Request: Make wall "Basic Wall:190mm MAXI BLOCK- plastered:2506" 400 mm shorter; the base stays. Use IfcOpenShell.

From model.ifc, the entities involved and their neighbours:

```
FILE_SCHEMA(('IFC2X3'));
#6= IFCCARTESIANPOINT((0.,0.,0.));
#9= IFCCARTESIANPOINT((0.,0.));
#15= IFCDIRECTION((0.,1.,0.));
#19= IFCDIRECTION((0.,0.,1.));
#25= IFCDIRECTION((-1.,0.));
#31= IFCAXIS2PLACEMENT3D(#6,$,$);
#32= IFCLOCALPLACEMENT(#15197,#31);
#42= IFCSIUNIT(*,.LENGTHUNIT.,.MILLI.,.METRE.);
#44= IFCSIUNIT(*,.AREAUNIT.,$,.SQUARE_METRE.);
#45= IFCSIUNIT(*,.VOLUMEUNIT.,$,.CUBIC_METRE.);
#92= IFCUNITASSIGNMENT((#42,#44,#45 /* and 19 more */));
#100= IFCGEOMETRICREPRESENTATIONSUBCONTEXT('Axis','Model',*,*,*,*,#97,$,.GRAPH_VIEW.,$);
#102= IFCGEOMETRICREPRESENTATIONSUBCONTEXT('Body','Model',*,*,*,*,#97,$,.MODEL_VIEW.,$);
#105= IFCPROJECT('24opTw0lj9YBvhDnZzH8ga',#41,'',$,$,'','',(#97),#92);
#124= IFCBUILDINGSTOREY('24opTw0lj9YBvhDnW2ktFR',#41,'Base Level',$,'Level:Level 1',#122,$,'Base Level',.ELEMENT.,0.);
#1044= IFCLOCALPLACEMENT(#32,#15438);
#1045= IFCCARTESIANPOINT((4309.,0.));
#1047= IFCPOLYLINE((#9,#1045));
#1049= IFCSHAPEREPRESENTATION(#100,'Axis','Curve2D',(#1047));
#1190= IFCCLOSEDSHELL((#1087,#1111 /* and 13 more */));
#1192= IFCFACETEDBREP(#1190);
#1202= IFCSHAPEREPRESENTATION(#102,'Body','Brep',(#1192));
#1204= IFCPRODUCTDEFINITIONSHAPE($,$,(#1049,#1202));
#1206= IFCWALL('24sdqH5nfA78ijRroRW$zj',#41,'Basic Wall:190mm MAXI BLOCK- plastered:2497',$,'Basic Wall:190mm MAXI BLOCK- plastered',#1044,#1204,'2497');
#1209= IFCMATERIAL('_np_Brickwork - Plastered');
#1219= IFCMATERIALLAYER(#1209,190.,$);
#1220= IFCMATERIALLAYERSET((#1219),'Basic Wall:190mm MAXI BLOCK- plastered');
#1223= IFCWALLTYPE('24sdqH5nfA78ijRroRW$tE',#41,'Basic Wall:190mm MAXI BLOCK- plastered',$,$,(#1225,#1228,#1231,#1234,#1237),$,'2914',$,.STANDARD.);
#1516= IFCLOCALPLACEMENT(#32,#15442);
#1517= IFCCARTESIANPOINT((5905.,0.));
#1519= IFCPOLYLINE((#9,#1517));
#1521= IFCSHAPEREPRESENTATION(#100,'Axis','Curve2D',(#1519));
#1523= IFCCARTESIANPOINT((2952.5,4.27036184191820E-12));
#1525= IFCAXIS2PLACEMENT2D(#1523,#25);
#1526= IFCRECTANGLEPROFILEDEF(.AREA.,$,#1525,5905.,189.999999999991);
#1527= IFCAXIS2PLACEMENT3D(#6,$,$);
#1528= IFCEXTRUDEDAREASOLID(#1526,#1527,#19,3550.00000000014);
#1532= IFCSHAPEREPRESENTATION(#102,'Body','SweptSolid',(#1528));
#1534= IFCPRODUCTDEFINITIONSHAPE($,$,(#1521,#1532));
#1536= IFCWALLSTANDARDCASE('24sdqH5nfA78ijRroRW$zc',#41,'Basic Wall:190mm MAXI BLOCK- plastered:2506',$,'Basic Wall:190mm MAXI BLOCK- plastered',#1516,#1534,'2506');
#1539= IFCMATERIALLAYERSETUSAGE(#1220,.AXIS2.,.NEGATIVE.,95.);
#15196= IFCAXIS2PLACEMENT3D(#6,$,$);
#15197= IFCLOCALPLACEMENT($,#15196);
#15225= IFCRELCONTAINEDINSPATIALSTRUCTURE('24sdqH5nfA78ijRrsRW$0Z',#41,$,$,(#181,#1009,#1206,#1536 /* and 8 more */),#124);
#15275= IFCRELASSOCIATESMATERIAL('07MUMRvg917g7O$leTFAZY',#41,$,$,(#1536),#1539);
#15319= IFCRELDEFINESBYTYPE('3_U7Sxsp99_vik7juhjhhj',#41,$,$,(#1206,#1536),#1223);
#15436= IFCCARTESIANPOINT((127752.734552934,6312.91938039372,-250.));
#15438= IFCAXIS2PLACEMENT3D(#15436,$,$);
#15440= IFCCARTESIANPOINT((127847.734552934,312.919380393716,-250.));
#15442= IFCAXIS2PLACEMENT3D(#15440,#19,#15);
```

```python
import ifcopenshell
import ifcopenshell.geom
import ifcopenshell.util.representation
import ifcopenshell.util.shape
import ifcopenshell.util.unit

model = ifcopenshell.open("model.ifc")
unit_scale = ifcopenshell.util.unit.calculate_unit_scale(model)
settings = ifcopenshell.geom.settings()


def volume(element):
    """Net volume in cubic metres, openings subtracted."""
    shape = ifcopenshell.geom.create_shape(settings, element)
    return ifcopenshell.util.shape.get_volume(shape.geometry)


wall = model.by_guid("24sdqH5nfA78ijRroRW$zc")
before = volume(wall)

body = ifcopenshell.util.representation.get_representation(wall, "Model", "Body")
solid = body.Items[0]
old_height = solid.Depth
solid.Depth -= 0.4 / unit_scale
after = volume(wall)

print(f"height {old_height:g} -> {solid.Depth:g}, volume {before:.3f} -> {after:.3f} m3")

model.write("model_v2.ifc")
```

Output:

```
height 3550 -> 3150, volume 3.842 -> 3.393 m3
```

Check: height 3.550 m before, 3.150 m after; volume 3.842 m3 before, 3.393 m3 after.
